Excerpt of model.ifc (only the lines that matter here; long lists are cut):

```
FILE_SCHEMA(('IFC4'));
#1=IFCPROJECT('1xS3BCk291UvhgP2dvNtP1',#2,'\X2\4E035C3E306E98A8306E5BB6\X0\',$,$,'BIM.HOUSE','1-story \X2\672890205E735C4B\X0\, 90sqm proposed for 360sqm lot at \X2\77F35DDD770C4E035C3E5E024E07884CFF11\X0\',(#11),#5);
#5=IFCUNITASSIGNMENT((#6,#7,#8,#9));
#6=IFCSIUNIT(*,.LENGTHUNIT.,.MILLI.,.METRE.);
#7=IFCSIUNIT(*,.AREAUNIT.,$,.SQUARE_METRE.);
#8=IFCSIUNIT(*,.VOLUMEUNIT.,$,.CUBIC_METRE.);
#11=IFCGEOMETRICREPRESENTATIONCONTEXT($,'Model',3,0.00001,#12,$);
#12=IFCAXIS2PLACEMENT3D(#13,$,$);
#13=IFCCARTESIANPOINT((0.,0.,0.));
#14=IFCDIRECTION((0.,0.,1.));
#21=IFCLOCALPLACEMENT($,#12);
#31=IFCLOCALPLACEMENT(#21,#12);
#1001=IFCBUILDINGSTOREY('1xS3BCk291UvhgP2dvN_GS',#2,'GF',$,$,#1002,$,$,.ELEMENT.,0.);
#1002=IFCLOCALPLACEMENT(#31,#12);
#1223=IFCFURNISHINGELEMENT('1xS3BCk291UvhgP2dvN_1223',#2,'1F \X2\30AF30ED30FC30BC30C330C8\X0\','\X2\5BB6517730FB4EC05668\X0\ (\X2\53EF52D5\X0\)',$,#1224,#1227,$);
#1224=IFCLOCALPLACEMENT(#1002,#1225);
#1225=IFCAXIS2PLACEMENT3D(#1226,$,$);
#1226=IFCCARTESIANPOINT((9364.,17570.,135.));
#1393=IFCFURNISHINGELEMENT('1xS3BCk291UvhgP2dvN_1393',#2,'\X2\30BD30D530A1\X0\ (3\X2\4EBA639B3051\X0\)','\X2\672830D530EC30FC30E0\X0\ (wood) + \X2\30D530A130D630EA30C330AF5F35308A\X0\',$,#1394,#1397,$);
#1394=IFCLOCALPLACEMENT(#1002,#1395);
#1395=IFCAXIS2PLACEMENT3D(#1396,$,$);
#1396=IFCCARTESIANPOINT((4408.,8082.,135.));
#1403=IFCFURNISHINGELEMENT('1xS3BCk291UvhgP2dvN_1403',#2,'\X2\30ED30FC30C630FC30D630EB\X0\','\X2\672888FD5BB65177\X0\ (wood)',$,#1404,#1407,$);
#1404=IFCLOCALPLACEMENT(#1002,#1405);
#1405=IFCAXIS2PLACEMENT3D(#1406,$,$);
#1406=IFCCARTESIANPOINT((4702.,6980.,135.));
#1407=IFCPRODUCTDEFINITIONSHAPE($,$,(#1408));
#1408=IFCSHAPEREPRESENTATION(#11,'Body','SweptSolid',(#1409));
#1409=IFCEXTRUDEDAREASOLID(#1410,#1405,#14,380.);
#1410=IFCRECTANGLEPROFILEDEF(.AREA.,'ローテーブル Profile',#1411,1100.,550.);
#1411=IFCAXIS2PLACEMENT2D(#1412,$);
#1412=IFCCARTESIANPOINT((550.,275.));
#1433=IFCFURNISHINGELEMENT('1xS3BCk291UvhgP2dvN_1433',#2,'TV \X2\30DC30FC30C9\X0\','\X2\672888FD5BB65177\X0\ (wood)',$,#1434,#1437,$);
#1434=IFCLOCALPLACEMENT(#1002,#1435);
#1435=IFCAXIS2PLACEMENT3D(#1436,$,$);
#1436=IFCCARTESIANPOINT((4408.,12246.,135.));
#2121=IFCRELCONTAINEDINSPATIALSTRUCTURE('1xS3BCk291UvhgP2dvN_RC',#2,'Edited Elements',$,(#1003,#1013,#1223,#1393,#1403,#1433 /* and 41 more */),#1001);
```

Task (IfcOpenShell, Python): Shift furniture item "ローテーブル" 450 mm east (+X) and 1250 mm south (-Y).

```python
import ifcopenshell
import ifcopenshell.api.geometry
import ifcopenshell.util.placement
import ifcopenshell.util.unit

model = ifcopenshell.open("model.ifc")
unit_scale = ifcopenshell.util.unit.calculate_unit_scale(model)

item = model.by_guid("1xS3BCk291UvhgP2dvN_1403")
matrix = ifcopenshell.util.placement.get_local_placement(item.ObjectPlacement)
matrix[0, 3] += 0.45 / unit_scale
matrix[1, 3] -= 1.25 / unit_scale
ifcopenshell.api.geometry.edit_object_placement(model, product=item, matrix=matrix, is_si=False)

print(ifcopenshell.util.placement.get_local_placement(item.ObjectPlacement).round(3) + 0.0)

model.write("model_rev.ifc")
```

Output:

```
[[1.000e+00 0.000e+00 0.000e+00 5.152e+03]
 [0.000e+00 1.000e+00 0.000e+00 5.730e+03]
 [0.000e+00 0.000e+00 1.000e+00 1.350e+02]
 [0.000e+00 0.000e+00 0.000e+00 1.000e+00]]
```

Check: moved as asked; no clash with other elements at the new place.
